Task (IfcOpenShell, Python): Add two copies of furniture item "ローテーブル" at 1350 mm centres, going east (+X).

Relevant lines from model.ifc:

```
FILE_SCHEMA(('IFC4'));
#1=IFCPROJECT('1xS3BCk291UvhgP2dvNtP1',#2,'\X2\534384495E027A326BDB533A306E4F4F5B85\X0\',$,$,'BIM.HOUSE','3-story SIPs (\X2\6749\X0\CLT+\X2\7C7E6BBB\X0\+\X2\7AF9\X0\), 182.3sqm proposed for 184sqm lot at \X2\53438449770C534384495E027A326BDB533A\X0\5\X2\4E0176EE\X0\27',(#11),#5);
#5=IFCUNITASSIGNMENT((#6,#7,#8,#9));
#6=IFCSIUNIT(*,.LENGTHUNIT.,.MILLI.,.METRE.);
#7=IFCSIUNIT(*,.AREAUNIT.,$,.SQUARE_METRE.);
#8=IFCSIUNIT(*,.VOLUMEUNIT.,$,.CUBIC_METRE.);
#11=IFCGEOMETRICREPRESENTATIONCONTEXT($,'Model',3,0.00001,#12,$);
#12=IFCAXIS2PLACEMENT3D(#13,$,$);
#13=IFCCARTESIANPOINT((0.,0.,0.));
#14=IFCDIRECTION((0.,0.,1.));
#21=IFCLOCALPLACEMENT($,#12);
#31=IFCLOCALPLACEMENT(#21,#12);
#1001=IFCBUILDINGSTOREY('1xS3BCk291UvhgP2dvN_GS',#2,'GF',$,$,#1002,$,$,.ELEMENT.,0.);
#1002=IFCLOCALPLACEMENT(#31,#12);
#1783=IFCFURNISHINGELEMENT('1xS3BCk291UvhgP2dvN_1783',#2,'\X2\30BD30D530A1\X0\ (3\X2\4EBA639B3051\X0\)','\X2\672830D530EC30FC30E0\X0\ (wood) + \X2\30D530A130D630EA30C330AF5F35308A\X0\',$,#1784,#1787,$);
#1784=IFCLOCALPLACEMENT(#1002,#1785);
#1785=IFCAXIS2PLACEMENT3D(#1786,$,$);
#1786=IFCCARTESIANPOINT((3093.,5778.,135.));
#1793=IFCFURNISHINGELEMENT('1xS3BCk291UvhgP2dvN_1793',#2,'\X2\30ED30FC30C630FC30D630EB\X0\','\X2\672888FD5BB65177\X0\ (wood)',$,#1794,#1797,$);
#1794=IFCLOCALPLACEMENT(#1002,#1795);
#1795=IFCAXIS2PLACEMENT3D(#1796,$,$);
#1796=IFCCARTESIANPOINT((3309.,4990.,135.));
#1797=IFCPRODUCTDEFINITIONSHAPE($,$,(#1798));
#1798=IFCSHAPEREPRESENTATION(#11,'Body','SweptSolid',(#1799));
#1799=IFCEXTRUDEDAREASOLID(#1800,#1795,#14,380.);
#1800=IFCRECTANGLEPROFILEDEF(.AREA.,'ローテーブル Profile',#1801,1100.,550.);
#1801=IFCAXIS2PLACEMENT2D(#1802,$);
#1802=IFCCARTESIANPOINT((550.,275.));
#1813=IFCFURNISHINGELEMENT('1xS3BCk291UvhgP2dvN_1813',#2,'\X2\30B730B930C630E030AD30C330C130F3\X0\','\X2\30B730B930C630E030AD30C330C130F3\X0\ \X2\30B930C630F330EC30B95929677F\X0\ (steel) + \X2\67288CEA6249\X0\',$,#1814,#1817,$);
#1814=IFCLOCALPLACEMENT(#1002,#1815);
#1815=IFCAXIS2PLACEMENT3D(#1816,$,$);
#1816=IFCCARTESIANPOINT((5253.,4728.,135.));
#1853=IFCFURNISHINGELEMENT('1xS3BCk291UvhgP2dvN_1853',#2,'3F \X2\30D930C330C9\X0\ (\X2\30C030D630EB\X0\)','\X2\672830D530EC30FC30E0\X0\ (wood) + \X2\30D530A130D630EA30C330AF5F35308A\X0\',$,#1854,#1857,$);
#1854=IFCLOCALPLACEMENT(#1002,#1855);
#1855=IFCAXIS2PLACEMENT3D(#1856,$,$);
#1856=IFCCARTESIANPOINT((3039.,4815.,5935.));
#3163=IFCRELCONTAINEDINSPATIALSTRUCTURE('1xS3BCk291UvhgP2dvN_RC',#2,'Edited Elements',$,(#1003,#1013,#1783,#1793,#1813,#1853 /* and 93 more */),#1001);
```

```python
import numpy as np
import ifcopenshell
import ifcopenshell.api.geometry
import ifcopenshell.api.root
import ifcopenshell.util.element
import ifcopenshell.util.placement
import ifcopenshell.util.unit

model = ifcopenshell.open("model.ifc")
unit_scale = ifcopenshell.util.unit.calculate_unit_scale(model)


def reuse_history(source, copy):
    """copy_class also copies each property set's owner history, people and application; keep the originals."""
    for rel in copy.IsDefinedBy:
        if rel.is_a("IfcRelDefinesByProperties") and (history := rel.RelatingPropertyDefinition.OwnerHistory):
            rel.RelatingPropertyDefinition.OwnerHistory = source.OwnerHistory
            ifcopenshell.util.element.remove_deep2(model, history)


source = model.by_id(1793)
base = ifcopenshell.util.placement.get_local_placement(source.ObjectPlacement)
step = np.array([1.0, 0.0, 0.0]) * 1.35 / unit_scale

for i in range(1, 3):
    copy = ifcopenshell.api.root.copy_class(model, product=source)
    copy.Representation = ifcopenshell.util.element.copy_deep(
        model, source.Representation, exclude=["IfcGeometricRepresentationContext", "IfcRepresentationMap"]
    )
    reuse_history(source, copy)
    matrix = base.copy()
    matrix[:3, 3] += i * step
    print("added at", matrix[:3, 3].round(3) + 0.0)
    ifcopenshell.api.geometry.edit_object_placement(model, product=copy, matrix=matrix, is_si=False)

model.write("model_v2.ifc")
```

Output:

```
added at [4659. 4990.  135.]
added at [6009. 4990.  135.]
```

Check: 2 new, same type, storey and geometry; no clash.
